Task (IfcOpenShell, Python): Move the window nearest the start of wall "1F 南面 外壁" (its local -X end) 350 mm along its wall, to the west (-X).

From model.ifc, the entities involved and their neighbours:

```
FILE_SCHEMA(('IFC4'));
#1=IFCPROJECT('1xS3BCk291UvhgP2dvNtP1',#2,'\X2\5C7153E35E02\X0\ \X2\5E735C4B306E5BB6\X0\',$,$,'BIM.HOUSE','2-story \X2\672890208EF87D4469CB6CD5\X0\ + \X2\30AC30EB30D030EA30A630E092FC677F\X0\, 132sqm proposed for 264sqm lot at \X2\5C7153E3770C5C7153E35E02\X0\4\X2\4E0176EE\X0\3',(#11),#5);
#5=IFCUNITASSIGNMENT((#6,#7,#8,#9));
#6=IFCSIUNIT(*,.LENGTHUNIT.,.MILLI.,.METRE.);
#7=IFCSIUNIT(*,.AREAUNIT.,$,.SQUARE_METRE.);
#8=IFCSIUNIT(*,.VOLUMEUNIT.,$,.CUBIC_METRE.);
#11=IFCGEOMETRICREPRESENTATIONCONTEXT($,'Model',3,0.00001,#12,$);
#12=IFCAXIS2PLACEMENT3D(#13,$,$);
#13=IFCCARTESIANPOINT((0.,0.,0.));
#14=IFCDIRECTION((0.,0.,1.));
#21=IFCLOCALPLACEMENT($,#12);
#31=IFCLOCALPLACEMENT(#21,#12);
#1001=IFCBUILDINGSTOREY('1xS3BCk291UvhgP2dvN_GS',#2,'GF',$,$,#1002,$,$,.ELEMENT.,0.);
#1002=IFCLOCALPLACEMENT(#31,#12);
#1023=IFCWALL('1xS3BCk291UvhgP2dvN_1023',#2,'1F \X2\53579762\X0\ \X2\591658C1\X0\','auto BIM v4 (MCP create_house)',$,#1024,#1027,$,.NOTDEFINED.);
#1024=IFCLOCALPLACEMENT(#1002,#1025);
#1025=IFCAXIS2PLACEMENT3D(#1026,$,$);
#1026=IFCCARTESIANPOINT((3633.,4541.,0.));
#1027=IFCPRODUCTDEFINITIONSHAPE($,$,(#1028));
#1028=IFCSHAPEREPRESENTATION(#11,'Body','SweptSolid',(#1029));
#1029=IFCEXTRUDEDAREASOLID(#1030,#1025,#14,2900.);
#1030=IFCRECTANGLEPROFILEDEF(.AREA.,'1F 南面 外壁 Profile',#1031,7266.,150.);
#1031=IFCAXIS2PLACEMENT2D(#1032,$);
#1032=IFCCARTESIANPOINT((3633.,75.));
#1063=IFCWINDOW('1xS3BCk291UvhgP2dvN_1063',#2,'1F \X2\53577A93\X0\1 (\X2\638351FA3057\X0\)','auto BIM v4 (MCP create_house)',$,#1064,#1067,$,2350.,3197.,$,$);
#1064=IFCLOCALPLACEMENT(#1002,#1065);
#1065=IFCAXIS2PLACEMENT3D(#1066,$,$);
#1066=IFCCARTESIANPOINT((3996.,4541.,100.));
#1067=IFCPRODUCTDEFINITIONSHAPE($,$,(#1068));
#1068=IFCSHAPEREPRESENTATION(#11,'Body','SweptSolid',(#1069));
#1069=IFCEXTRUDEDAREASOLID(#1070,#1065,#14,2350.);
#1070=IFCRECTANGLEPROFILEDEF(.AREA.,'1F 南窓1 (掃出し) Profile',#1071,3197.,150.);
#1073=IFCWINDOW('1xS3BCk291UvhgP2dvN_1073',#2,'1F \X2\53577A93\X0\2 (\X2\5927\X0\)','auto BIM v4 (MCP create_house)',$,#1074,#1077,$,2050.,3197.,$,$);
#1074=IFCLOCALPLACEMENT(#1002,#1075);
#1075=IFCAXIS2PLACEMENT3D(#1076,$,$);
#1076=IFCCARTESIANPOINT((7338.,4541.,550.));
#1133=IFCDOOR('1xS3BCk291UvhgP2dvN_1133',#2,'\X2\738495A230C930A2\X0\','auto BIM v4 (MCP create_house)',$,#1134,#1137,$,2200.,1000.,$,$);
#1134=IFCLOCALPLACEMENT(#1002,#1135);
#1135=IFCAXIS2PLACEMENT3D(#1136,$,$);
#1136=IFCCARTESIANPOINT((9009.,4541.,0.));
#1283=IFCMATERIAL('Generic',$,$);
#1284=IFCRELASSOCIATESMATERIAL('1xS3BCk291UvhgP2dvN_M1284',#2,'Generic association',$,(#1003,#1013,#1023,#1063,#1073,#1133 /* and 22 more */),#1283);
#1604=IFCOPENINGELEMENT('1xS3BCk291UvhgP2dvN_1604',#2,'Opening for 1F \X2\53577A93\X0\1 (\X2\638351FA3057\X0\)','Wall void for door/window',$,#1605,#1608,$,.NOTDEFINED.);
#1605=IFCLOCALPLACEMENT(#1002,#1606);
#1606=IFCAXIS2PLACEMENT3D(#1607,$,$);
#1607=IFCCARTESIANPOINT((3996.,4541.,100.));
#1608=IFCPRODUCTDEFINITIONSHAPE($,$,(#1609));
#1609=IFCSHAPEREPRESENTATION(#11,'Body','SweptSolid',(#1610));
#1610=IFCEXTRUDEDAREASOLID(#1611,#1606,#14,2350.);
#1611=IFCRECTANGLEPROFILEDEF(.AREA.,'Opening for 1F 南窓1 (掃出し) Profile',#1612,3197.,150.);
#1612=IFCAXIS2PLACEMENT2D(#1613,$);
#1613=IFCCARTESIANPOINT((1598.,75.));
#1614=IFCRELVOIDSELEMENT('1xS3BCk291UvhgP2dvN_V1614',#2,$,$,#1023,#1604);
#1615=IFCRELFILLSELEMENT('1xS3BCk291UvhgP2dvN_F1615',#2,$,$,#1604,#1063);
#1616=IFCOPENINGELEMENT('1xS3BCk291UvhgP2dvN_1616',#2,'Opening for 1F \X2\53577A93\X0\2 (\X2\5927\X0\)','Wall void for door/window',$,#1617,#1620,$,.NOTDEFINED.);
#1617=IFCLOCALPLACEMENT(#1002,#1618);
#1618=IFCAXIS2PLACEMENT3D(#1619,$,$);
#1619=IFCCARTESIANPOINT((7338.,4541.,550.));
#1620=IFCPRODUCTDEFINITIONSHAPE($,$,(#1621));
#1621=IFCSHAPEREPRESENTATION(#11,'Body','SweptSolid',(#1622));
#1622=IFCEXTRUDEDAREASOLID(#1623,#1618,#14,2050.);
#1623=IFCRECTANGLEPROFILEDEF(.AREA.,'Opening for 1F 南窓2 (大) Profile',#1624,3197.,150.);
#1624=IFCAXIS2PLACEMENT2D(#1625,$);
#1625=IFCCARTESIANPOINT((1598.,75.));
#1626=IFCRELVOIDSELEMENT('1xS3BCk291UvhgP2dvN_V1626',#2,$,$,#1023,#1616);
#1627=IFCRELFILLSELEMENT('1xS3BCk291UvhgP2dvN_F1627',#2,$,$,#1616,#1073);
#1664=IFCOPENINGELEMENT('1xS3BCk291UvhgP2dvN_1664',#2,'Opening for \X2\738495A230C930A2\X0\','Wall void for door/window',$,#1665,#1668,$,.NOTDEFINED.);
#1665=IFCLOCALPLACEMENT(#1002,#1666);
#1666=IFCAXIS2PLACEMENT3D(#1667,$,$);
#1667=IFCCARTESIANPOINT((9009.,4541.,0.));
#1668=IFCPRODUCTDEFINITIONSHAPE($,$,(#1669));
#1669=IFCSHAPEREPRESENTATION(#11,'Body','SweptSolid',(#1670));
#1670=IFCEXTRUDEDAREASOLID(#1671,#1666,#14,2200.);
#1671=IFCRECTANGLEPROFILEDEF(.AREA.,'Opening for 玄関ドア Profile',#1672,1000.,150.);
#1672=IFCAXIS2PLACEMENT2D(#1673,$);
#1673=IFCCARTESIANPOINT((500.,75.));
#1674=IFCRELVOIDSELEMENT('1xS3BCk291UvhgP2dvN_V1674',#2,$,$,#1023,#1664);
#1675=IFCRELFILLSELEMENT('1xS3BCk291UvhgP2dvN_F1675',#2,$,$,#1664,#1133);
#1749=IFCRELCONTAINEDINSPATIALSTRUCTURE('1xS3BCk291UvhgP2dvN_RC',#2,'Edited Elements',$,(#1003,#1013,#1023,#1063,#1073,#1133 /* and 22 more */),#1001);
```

```python
import ifcopenshell
import ifcopenshell.api.geometry
import ifcopenshell.util.placement

model = ifcopenshell.open("model.ifc")

window = model.by_guid("1xS3BCk291UvhgP2dvN_1063")
opening = window.FillsVoids[0].RelatingOpeningElement
wall = opening.VoidsElements[0].RelatingBuildingElement

wall_matrix = ifcopenshell.util.placement.get_local_placement(wall.ObjectPlacement)
shift = wall_matrix[:3, 0] * -350.0
before = ifcopenshell.util.placement.get_local_placement(window.ObjectPlacement)[:3, 3].copy()

# The window is not placed relative to its opening, so move both.
for product in (opening, window):
    matrix = ifcopenshell.util.placement.get_local_placement(product.ObjectPlacement)
    matrix[:3, 3] += shift
    ifcopenshell.api.geometry.edit_object_placement(model, product=product, matrix=matrix, is_si=False)

after = ifcopenshell.util.placement.get_local_placement(window.ObjectPlacement)[:3, 3]
print("window moved by", (after - before).round(3) + 0.0)

model.write("model-out.ifc")
```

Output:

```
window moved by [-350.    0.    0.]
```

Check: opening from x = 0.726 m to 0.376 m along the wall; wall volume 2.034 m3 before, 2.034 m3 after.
